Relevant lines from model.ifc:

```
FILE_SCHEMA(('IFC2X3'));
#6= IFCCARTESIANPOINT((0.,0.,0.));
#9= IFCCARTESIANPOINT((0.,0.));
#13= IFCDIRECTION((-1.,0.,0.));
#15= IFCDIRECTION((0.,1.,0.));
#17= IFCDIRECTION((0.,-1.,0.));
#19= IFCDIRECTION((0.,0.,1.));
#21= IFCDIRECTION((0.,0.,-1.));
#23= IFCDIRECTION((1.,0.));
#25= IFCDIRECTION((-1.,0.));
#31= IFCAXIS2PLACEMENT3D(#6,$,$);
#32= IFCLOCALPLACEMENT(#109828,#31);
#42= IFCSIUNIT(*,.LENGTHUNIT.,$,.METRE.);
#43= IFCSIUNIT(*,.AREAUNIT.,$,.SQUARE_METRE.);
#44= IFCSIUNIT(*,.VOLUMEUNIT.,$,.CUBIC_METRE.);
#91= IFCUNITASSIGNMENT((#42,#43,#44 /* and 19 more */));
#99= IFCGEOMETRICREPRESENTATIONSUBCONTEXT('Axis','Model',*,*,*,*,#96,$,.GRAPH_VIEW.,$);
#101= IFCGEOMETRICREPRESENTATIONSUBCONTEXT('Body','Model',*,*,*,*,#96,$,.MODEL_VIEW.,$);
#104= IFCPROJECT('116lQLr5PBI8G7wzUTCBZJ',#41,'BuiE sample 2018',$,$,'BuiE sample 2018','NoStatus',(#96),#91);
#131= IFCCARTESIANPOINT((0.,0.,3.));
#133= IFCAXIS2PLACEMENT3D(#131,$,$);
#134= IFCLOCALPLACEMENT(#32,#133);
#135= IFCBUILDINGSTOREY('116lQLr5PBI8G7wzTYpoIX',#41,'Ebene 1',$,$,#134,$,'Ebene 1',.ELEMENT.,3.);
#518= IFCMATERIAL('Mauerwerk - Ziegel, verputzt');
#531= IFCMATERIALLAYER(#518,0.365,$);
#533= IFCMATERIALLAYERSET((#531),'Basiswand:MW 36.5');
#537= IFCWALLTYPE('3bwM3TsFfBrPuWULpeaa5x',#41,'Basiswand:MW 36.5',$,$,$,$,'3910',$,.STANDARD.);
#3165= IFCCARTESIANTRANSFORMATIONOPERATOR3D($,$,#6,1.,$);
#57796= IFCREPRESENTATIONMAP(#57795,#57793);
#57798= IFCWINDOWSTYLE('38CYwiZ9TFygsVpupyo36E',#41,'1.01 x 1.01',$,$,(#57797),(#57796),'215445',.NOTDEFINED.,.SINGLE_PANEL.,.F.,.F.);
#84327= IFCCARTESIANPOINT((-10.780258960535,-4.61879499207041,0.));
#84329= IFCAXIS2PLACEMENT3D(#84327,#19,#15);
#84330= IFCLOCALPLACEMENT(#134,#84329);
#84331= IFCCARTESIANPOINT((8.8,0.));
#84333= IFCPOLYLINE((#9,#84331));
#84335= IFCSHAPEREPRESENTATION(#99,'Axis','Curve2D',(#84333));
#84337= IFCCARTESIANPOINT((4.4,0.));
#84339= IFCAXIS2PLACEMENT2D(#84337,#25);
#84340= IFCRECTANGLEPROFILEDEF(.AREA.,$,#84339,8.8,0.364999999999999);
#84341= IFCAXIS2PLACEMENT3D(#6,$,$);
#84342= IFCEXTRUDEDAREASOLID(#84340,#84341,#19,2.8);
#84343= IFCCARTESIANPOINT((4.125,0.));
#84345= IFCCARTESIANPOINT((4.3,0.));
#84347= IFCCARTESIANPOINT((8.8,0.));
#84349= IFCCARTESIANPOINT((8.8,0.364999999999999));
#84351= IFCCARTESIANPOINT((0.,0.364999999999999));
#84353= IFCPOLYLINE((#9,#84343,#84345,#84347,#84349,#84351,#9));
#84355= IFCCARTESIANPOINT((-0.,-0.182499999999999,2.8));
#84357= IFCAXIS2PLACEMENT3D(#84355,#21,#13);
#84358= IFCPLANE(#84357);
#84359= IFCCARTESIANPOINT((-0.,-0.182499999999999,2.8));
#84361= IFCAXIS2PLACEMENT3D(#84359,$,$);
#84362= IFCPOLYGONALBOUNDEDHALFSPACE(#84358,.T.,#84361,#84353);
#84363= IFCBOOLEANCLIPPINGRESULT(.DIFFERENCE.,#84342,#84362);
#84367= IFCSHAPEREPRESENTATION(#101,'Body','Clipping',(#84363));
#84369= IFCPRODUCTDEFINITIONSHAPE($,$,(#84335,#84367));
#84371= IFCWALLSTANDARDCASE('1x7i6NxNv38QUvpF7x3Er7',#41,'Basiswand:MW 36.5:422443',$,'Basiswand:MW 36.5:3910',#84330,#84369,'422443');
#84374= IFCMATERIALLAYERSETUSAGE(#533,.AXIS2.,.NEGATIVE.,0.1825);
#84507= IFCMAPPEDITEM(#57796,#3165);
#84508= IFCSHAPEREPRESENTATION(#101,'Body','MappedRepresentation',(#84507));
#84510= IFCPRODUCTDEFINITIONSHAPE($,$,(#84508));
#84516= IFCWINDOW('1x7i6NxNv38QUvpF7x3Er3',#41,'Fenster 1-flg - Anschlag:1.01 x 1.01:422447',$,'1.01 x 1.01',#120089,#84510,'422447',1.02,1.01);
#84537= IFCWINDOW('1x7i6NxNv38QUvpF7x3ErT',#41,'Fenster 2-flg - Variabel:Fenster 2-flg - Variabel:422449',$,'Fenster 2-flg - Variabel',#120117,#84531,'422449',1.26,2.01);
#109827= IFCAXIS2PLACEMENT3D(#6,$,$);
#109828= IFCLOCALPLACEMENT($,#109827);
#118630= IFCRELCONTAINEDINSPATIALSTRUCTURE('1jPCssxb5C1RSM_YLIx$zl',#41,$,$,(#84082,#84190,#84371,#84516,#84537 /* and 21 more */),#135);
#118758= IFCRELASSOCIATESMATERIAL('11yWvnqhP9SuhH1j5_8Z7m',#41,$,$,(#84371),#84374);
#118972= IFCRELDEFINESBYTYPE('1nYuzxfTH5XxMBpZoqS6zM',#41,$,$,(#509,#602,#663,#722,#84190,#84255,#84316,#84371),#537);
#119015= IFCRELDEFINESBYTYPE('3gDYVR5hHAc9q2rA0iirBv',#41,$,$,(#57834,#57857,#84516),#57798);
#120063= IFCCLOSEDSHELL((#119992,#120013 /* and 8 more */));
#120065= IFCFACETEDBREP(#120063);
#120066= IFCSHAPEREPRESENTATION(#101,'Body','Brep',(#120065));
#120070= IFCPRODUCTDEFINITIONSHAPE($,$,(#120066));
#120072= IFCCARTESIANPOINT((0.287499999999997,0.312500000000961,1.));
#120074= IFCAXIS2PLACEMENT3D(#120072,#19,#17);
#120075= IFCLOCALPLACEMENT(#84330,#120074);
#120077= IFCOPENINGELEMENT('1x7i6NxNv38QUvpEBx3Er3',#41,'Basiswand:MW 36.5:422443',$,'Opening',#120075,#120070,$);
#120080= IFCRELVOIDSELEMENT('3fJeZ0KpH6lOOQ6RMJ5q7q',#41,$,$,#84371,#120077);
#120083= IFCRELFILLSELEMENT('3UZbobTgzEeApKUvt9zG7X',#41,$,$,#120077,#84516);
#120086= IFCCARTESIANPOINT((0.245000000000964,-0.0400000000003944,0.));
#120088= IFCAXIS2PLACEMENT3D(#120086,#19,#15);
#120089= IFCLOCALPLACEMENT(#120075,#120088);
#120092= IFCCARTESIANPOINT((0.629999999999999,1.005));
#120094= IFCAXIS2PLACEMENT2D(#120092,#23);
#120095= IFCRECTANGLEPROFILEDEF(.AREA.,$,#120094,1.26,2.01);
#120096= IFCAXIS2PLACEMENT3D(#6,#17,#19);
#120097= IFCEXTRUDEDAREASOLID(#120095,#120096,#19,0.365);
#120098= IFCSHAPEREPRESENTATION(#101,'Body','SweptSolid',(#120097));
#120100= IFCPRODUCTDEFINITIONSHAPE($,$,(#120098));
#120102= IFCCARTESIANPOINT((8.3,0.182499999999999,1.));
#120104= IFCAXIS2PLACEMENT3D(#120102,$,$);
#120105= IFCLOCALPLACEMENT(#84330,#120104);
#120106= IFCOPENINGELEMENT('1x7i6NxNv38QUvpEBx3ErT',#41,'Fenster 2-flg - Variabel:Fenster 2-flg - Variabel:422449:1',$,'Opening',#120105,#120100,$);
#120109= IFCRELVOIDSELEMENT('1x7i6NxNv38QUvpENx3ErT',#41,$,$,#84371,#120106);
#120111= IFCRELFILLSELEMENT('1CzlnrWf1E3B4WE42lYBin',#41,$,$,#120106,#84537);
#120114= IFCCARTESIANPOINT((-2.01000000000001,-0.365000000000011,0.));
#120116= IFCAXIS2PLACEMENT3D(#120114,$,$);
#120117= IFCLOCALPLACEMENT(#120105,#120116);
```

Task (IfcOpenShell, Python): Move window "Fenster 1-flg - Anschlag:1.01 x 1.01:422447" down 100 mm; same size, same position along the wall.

```python
import numpy as np
import ifcopenshell
import ifcopenshell.api.geometry
import ifcopenshell.util.placement
import ifcopenshell.util.unit

model = ifcopenshell.open("model.ifc")
unit_scale = ifcopenshell.util.unit.calculate_unit_scale(model)

window = model.by_guid("1x7i6NxNv38QUvpF7x3Er3")
opening = window.FillsVoids[0].RelatingOpeningElement
dz = -0.1

shift = np.array([0.0, 0.0, dz])
# The window is placed relative to its opening, so it follows when the opening moves.
matrix = ifcopenshell.util.placement.get_local_placement(opening.ObjectPlacement)
matrix[:3, 3] += shift
ifcopenshell.api.geometry.edit_object_placement(
    model, product=opening, matrix=matrix, is_si=False, should_transform_children=True
)

print(f"moved by {dz * unit_scale:+.3f} m")

model.write("model_edited.ifc")
```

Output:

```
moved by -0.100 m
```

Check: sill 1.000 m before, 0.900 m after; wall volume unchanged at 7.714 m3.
